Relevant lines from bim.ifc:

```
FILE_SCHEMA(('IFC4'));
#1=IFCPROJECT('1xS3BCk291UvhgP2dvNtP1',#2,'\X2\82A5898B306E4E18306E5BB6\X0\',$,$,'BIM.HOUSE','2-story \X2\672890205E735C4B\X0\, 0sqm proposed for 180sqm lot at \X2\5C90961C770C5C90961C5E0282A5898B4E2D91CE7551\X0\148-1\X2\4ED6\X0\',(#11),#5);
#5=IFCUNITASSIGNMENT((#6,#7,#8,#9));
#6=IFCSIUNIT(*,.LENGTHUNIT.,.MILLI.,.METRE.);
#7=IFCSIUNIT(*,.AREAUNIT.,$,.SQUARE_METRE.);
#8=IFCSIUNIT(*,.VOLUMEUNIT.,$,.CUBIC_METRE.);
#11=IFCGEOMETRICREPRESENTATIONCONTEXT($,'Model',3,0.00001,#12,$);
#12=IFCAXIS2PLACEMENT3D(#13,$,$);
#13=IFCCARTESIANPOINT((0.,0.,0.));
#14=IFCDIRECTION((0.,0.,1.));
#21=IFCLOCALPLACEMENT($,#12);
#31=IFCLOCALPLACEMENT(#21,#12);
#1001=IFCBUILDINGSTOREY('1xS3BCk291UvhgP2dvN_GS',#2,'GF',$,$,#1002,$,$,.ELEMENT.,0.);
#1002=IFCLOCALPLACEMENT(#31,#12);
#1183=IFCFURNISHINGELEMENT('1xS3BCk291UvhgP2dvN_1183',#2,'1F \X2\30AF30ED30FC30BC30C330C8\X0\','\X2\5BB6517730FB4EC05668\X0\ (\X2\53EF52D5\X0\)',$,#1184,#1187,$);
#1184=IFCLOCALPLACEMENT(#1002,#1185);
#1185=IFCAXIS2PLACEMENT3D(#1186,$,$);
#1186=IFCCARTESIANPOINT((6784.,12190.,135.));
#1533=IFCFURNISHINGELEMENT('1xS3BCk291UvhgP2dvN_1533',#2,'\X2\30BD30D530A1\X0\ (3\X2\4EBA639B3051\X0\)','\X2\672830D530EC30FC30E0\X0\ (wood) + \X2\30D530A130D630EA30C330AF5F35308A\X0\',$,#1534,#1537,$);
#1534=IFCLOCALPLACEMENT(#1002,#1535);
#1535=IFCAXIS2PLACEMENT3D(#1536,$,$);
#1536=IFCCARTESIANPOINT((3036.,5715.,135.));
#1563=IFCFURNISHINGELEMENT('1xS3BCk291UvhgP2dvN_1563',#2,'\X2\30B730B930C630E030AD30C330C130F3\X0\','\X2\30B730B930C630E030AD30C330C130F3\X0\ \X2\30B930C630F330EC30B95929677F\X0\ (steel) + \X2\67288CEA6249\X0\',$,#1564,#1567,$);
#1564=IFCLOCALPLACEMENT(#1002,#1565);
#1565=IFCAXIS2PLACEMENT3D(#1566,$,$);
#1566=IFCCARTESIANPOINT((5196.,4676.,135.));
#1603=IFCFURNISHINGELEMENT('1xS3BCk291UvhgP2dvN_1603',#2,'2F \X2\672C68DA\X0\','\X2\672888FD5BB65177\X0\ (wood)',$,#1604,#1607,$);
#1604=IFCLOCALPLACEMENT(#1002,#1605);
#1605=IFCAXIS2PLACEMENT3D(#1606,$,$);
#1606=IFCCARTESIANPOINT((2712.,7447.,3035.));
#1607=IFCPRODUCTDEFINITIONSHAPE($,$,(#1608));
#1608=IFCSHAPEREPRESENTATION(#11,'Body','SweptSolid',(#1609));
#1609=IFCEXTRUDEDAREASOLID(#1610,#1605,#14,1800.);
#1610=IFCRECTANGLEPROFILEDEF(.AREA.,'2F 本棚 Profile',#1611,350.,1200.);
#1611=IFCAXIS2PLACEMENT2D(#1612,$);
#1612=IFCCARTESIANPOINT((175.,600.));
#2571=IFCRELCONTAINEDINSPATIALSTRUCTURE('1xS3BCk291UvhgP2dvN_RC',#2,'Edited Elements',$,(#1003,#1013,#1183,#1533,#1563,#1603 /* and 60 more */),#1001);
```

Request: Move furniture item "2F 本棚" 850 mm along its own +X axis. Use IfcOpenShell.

```python
import ifcopenshell
import ifcopenshell.api.geometry
import ifcopenshell.util.placement
import ifcopenshell.util.unit

model = ifcopenshell.open("bim.ifc")
unit_scale = ifcopenshell.util.unit.calculate_unit_scale(model)

item = model.by_id(1603)
matrix = ifcopenshell.util.placement.get_local_placement(item.ObjectPlacement)
matrix[:3, 3] += matrix[:3, 0] * 0.85 / unit_scale
ifcopenshell.api.geometry.edit_object_placement(model, product=item, matrix=matrix, is_si=False)

print(ifcopenshell.util.placement.get_local_placement(item.ObjectPlacement).round(3) + 0.0)

model.write("bim_rev.ifc")
```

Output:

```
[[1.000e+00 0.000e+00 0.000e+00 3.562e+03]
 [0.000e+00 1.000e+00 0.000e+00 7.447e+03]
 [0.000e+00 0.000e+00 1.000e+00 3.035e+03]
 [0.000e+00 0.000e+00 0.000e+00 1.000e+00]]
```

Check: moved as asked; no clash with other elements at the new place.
